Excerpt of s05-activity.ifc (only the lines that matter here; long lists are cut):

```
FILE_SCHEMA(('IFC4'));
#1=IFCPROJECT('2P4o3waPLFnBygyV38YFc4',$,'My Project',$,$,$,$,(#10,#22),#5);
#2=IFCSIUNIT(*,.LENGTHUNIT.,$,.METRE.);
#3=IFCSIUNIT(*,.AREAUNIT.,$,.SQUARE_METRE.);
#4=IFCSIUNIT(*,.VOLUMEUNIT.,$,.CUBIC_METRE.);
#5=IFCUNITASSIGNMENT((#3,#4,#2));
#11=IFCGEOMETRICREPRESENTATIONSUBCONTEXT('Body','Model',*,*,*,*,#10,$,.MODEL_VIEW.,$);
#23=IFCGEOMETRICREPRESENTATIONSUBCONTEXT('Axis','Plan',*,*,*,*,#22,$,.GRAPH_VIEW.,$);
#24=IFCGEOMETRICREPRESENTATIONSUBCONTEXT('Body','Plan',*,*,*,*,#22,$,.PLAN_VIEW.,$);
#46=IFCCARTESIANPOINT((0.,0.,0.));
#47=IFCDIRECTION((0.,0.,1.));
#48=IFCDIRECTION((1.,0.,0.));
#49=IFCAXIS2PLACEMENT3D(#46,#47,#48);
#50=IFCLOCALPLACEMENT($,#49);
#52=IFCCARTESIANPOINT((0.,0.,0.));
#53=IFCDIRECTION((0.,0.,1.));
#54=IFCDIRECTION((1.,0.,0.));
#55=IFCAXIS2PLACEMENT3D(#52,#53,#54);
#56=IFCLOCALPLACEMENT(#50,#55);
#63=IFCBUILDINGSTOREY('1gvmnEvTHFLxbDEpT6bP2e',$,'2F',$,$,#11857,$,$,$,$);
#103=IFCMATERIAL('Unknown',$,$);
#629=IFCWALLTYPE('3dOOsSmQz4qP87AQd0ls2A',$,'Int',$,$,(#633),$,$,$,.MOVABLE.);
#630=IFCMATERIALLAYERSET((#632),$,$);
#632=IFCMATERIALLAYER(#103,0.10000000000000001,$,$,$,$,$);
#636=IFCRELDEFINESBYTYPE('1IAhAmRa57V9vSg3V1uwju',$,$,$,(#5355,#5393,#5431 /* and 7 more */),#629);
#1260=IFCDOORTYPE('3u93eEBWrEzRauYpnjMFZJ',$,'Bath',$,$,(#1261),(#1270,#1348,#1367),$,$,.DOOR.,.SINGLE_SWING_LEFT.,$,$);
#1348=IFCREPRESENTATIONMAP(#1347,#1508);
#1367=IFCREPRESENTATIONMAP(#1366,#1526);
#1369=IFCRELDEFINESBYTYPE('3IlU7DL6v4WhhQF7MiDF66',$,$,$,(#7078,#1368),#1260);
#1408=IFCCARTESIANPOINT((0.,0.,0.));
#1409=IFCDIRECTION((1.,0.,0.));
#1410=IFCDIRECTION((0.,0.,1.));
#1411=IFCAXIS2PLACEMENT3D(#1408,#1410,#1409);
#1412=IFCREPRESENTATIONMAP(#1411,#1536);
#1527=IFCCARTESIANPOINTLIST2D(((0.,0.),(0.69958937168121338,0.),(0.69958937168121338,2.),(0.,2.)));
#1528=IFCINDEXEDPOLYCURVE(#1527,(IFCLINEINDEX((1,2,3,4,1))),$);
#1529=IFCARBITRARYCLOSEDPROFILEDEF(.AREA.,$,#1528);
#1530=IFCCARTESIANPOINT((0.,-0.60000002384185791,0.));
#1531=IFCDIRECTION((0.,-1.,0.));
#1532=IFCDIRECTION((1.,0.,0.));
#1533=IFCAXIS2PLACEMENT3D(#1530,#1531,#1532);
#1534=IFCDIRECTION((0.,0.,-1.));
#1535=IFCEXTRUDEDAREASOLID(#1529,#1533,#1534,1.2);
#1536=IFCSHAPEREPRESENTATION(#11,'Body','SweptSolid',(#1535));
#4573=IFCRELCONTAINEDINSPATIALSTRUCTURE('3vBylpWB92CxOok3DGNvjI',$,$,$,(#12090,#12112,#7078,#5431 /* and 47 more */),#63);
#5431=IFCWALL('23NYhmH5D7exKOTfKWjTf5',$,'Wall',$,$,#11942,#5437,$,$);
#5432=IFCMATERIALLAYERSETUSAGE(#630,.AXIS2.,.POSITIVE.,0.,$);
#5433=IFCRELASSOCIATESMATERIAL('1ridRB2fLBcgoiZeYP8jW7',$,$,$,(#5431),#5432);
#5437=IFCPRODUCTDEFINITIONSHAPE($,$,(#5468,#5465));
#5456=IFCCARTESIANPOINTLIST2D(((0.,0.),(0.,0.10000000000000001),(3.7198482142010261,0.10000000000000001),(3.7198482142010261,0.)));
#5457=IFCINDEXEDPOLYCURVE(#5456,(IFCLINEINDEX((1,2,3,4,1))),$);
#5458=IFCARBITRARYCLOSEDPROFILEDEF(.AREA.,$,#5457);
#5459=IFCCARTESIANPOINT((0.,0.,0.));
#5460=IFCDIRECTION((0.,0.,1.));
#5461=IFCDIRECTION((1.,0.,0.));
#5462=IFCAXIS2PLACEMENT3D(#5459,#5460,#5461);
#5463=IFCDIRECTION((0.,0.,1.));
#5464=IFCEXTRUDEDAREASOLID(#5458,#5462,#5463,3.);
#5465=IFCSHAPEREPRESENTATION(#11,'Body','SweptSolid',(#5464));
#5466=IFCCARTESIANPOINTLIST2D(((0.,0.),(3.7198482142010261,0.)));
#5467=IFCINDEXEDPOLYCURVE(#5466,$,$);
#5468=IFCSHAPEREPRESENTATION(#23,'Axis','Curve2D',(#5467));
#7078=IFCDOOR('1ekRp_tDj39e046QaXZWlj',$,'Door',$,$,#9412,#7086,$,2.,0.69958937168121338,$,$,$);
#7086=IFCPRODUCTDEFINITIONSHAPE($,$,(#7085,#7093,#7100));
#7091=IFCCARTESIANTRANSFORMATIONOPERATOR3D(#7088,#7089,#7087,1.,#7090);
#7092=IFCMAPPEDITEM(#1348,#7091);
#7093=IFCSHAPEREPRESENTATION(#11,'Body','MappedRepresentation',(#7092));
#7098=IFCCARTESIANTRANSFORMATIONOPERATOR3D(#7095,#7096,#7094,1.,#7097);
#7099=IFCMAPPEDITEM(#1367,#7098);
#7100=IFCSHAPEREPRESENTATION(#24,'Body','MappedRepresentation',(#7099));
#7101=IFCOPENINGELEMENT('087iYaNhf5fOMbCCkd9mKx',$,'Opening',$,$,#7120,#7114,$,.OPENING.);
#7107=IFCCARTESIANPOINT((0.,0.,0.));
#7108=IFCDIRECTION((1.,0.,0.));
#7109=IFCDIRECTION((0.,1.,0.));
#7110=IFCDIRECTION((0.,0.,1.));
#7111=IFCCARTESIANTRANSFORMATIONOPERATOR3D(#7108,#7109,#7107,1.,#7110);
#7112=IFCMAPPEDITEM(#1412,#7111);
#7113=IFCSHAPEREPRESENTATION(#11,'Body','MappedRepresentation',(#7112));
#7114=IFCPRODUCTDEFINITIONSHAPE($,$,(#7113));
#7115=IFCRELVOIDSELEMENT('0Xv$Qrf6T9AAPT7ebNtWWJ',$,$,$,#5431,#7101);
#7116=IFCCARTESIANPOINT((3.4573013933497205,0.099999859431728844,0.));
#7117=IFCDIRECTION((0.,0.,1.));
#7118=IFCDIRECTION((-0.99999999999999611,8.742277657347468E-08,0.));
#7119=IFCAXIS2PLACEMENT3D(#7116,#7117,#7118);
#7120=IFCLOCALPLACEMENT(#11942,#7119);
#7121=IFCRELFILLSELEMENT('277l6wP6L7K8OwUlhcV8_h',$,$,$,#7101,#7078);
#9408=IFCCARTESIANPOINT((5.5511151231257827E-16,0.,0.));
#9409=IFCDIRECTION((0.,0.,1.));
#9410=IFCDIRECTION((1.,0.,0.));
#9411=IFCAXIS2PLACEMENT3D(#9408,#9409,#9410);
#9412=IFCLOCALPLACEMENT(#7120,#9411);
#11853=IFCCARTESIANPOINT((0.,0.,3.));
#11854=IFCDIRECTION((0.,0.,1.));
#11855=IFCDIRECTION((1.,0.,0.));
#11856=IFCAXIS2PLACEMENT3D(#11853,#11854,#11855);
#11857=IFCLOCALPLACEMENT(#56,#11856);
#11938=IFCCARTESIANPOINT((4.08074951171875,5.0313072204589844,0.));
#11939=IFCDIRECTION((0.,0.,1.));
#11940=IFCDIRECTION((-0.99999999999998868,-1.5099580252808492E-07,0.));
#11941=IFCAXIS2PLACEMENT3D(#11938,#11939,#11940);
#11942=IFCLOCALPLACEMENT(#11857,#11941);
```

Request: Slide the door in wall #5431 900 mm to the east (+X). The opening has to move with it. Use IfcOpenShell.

```python
import ifcopenshell
import ifcopenshell.api.geometry
import ifcopenshell.util.placement

model = ifcopenshell.open("s05-activity.ifc")

door = model.by_guid("1ekRp_tDj39e046QaXZWlj")
opening = door.FillsVoids[0].RelatingOpeningElement
wall = opening.VoidsElements[0].RelatingBuildingElement

wall_matrix = ifcopenshell.util.placement.get_local_placement(wall.ObjectPlacement)
shift = wall_matrix[:3, 0] * -0.9
before = ifcopenshell.util.placement.get_local_placement(door.ObjectPlacement)[:3, 3].copy()

# The door is placed relative to its opening, so it follows when the opening moves.
matrix = ifcopenshell.util.placement.get_local_placement(opening.ObjectPlacement)
matrix[:3, 3] += shift
ifcopenshell.api.geometry.edit_object_placement(
    model, product=opening, matrix=matrix, is_si=False, should_transform_children=True
)

after = ifcopenshell.util.placement.get_local_placement(door.ObjectPlacement)[:3, 3]
print("door moved by", (after - before).round(3) + 0.0)

model.write("s05-activity_edited.ifc")
```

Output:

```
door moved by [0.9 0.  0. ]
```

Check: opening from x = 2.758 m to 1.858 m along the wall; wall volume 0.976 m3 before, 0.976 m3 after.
